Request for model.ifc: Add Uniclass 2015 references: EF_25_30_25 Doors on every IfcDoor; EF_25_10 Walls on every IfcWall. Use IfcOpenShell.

First a look at what the model holds.

```python
import ifcopenshell

model = ifcopenshell.open("model.ifc")
print(model.schema)
print("classifications:", [c.Name for c in model.by_type("IfcClassification")])
for ifc_class in ("IfcDoor", "IfcRoof", "IfcStair", "IfcWall", "IfcWindow"):
    print(ifc_class, len(model.by_type(ifc_class)))
```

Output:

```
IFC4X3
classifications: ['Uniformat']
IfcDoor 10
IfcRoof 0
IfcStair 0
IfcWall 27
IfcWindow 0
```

```python
import ifcopenshell
import ifcopenshell.api.classification

model = ifcopenshell.open("model.ifc")

system = ifcopenshell.api.classification.add_classification(model, classification="Uniclass 2015")

codes = {
    "IfcDoor": ("EF_25_30_25", "Doors"),
    "IfcWall": ("EF_25_10", "Walls"),
}
for ifc_class, (code, name) in codes.items():
    products = model.by_type(ifc_class)
    ifcopenshell.api.classification.add_reference(
        model, products=products, classification=system, identification=code, name=name
    )
    print(code, len(products))

model.write("model_updated.ifc")
```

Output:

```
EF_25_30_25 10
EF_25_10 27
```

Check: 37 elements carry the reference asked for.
